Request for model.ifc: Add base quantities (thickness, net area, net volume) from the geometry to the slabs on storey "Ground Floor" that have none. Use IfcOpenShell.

First a look at what the model holds.

```python
import ifcopenshell
import ifcopenshell.util.element
import ifcopenshell.util.unit

model = ifcopenshell.open("model.ifc")
print(model.schema)
for unit_type in ("LENGTHUNIT", "AREAUNIT", "VOLUMEUNIT"):
    print(unit_type, ifcopenshell.util.unit.calculate_unit_scale(model, unit_type))
storey = next(s for s in model.by_type("IfcBuildingStorey") if s.Name == "Ground Floor")
slabs = [e for e in ifcopenshell.util.element.get_decomposition(storey) if e.is_a("IfcSlab")]
for e in sorted(slabs, key=lambda e: e.id()):
    print(e.id(), e.is_a(), e.Name, list(ifcopenshell.util.element.get_psets(e, qtos_only=True)), sep=" | ")
```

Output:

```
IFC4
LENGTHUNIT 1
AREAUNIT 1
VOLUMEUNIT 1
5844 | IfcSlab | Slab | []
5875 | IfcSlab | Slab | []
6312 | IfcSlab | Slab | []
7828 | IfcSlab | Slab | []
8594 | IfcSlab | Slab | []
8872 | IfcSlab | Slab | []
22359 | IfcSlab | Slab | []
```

```python
import ifcopenshell
import ifcopenshell.api.pset
import ifcopenshell.geom
import ifcopenshell.util.element
import ifcopenshell.util.shape
import ifcopenshell.util.unit

model = ifcopenshell.open("model.ifc")
unit_scale = ifcopenshell.util.unit.calculate_unit_scale(model)
area_scale = ifcopenshell.util.unit.calculate_unit_scale(model, "AREAUNIT")
volume_scale = ifcopenshell.util.unit.calculate_unit_scale(model, "VOLUMEUNIT")
settings = ifcopenshell.geom.settings()

storey = next(s for s in model.by_type("IfcBuildingStorey") if s.Name == "Ground Floor")
slabs = [e for e in ifcopenshell.util.element.get_decomposition(storey) if e.is_a("IfcSlab")]

for e in sorted(slabs, key=lambda e: e.id()):
    if ifcopenshell.util.element.get_psets(e, qtos_only=True, should_inherit=False):
        continue
    # Geometry comes back in metres, in the element's own axes.
    shape = ifcopenshell.geom.create_shape(settings, e)
    values = {
        "Width": ifcopenshell.util.shape.get_z(shape.geometry) / unit_scale,
        "NetArea": ifcopenshell.util.shape.get_footprint_area(shape.geometry) / area_scale,
        "NetVolume": ifcopenshell.util.shape.get_volume(shape.geometry) / volume_scale,
    }
    qto = ifcopenshell.api.pset.add_qto(model, product=e, name="Qto_SlabBaseQuantities")
    ifcopenshell.api.pset.edit_qto(model, qto=qto, properties=values)
    print(e.id(), {k: round(v, 3) for k, v in values.items()})

model.write("model_rev.ifc")
```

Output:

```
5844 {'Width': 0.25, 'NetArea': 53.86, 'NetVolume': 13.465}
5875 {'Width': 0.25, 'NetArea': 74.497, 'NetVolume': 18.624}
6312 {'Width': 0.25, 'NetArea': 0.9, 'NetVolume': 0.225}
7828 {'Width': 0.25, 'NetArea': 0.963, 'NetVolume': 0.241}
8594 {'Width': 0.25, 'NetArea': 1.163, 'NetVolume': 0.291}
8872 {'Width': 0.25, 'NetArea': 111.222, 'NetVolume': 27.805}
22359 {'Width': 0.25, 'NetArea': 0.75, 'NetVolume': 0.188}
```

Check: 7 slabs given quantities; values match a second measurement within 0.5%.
